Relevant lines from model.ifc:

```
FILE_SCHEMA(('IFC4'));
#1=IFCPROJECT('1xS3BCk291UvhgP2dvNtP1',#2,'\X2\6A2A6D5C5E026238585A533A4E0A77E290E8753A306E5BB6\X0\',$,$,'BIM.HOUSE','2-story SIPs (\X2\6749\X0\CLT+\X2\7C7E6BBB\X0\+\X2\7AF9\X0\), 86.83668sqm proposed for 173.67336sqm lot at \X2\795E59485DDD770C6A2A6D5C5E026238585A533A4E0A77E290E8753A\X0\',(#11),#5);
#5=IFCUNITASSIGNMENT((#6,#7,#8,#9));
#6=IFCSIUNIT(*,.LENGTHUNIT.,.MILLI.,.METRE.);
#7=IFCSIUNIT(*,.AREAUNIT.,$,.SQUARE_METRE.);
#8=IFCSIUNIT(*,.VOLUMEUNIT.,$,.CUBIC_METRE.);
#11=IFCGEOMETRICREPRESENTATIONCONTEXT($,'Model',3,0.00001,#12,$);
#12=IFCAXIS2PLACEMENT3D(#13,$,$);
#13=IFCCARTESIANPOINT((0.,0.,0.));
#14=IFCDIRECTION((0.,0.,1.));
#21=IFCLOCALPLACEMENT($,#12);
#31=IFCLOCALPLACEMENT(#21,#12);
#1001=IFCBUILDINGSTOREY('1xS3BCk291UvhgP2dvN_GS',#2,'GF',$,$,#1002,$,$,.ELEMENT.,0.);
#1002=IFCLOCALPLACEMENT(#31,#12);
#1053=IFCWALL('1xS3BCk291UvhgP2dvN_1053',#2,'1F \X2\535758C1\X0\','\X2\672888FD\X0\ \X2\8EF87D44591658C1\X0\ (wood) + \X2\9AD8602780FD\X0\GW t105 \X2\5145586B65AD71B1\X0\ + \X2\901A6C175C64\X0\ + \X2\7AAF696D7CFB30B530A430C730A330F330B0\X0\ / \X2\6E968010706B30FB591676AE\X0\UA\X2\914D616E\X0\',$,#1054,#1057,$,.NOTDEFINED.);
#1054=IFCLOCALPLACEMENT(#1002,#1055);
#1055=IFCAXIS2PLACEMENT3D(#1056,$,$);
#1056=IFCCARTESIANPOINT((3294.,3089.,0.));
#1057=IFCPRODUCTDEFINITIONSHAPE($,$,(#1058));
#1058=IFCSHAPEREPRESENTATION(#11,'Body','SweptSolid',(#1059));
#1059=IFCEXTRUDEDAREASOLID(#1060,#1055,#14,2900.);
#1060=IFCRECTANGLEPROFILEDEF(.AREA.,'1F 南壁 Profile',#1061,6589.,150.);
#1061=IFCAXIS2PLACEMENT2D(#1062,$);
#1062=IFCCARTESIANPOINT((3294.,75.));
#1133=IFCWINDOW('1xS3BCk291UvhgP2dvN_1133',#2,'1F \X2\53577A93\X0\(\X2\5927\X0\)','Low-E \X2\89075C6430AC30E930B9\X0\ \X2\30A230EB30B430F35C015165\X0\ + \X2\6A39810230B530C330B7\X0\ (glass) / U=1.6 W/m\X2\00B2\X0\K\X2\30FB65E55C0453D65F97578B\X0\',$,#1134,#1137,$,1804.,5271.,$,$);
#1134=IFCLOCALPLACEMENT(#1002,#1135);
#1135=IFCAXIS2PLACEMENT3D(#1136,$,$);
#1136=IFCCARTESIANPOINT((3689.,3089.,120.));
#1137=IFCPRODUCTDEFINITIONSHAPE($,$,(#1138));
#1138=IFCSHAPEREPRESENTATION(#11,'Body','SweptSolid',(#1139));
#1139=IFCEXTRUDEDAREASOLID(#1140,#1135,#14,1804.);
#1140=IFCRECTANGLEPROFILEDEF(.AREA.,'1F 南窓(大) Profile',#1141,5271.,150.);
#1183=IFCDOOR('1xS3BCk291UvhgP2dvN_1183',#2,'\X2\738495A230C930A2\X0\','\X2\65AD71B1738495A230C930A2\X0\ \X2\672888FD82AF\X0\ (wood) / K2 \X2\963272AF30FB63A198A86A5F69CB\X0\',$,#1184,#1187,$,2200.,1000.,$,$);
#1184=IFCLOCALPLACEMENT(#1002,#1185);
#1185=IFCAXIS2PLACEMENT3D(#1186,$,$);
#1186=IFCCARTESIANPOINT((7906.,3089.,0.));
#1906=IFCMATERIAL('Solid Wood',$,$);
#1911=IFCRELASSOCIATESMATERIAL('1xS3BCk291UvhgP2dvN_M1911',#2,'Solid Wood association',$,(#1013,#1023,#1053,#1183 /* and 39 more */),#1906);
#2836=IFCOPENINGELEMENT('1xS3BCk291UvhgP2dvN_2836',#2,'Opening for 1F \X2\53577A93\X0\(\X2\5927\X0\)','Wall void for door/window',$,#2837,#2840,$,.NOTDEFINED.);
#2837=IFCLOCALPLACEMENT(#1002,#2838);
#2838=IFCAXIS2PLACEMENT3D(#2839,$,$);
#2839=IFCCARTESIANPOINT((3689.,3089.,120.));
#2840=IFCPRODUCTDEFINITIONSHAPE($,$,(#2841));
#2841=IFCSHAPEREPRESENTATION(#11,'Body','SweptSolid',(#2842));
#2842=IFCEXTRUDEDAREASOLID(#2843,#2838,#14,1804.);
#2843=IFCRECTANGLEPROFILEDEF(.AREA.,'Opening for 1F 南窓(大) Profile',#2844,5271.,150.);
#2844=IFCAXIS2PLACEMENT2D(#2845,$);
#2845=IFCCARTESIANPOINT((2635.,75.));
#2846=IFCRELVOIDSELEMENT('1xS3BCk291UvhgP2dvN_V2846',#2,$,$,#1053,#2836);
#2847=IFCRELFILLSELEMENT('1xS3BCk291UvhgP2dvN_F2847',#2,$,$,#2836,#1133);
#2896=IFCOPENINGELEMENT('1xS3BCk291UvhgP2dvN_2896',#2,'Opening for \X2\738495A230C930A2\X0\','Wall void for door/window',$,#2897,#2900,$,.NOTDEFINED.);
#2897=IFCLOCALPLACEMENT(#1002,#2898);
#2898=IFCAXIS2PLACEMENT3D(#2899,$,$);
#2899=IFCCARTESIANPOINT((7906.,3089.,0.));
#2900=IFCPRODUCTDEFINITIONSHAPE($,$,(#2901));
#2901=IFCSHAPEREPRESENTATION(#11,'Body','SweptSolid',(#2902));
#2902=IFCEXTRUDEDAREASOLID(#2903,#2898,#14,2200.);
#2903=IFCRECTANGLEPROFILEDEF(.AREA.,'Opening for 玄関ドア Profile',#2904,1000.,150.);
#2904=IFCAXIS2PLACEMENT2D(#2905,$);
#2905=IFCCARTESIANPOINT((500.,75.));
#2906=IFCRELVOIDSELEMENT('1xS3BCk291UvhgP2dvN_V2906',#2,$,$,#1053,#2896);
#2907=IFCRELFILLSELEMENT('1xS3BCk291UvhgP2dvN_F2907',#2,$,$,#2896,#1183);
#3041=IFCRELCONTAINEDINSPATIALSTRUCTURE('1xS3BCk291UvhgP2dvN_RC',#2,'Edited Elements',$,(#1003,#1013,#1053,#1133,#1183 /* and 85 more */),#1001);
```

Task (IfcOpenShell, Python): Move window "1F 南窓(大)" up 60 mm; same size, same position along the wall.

```python
import numpy as np
import ifcopenshell
import ifcopenshell.api.geometry
import ifcopenshell.util.placement
import ifcopenshell.util.unit

model = ifcopenshell.open("model.ifc")
unit_scale = ifcopenshell.util.unit.calculate_unit_scale(model)

window = model.by_guid("1xS3BCk291UvhgP2dvN_1133")
opening = window.FillsVoids[0].RelatingOpeningElement
dz = 0.06 / unit_scale

shift = np.array([0.0, 0.0, dz])
# The window is not placed relative to its opening, so move both.
for product in (opening, window):
    matrix = ifcopenshell.util.placement.get_local_placement(product.ObjectPlacement)
    matrix[:3, 3] += shift
    ifcopenshell.api.geometry.edit_object_placement(model, product=product, matrix=matrix, is_si=False)

print(f"moved by {dz * unit_scale:+.3f} m")

model.write("model_updated.ifc")
```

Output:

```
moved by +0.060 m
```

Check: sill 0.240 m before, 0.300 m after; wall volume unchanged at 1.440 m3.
